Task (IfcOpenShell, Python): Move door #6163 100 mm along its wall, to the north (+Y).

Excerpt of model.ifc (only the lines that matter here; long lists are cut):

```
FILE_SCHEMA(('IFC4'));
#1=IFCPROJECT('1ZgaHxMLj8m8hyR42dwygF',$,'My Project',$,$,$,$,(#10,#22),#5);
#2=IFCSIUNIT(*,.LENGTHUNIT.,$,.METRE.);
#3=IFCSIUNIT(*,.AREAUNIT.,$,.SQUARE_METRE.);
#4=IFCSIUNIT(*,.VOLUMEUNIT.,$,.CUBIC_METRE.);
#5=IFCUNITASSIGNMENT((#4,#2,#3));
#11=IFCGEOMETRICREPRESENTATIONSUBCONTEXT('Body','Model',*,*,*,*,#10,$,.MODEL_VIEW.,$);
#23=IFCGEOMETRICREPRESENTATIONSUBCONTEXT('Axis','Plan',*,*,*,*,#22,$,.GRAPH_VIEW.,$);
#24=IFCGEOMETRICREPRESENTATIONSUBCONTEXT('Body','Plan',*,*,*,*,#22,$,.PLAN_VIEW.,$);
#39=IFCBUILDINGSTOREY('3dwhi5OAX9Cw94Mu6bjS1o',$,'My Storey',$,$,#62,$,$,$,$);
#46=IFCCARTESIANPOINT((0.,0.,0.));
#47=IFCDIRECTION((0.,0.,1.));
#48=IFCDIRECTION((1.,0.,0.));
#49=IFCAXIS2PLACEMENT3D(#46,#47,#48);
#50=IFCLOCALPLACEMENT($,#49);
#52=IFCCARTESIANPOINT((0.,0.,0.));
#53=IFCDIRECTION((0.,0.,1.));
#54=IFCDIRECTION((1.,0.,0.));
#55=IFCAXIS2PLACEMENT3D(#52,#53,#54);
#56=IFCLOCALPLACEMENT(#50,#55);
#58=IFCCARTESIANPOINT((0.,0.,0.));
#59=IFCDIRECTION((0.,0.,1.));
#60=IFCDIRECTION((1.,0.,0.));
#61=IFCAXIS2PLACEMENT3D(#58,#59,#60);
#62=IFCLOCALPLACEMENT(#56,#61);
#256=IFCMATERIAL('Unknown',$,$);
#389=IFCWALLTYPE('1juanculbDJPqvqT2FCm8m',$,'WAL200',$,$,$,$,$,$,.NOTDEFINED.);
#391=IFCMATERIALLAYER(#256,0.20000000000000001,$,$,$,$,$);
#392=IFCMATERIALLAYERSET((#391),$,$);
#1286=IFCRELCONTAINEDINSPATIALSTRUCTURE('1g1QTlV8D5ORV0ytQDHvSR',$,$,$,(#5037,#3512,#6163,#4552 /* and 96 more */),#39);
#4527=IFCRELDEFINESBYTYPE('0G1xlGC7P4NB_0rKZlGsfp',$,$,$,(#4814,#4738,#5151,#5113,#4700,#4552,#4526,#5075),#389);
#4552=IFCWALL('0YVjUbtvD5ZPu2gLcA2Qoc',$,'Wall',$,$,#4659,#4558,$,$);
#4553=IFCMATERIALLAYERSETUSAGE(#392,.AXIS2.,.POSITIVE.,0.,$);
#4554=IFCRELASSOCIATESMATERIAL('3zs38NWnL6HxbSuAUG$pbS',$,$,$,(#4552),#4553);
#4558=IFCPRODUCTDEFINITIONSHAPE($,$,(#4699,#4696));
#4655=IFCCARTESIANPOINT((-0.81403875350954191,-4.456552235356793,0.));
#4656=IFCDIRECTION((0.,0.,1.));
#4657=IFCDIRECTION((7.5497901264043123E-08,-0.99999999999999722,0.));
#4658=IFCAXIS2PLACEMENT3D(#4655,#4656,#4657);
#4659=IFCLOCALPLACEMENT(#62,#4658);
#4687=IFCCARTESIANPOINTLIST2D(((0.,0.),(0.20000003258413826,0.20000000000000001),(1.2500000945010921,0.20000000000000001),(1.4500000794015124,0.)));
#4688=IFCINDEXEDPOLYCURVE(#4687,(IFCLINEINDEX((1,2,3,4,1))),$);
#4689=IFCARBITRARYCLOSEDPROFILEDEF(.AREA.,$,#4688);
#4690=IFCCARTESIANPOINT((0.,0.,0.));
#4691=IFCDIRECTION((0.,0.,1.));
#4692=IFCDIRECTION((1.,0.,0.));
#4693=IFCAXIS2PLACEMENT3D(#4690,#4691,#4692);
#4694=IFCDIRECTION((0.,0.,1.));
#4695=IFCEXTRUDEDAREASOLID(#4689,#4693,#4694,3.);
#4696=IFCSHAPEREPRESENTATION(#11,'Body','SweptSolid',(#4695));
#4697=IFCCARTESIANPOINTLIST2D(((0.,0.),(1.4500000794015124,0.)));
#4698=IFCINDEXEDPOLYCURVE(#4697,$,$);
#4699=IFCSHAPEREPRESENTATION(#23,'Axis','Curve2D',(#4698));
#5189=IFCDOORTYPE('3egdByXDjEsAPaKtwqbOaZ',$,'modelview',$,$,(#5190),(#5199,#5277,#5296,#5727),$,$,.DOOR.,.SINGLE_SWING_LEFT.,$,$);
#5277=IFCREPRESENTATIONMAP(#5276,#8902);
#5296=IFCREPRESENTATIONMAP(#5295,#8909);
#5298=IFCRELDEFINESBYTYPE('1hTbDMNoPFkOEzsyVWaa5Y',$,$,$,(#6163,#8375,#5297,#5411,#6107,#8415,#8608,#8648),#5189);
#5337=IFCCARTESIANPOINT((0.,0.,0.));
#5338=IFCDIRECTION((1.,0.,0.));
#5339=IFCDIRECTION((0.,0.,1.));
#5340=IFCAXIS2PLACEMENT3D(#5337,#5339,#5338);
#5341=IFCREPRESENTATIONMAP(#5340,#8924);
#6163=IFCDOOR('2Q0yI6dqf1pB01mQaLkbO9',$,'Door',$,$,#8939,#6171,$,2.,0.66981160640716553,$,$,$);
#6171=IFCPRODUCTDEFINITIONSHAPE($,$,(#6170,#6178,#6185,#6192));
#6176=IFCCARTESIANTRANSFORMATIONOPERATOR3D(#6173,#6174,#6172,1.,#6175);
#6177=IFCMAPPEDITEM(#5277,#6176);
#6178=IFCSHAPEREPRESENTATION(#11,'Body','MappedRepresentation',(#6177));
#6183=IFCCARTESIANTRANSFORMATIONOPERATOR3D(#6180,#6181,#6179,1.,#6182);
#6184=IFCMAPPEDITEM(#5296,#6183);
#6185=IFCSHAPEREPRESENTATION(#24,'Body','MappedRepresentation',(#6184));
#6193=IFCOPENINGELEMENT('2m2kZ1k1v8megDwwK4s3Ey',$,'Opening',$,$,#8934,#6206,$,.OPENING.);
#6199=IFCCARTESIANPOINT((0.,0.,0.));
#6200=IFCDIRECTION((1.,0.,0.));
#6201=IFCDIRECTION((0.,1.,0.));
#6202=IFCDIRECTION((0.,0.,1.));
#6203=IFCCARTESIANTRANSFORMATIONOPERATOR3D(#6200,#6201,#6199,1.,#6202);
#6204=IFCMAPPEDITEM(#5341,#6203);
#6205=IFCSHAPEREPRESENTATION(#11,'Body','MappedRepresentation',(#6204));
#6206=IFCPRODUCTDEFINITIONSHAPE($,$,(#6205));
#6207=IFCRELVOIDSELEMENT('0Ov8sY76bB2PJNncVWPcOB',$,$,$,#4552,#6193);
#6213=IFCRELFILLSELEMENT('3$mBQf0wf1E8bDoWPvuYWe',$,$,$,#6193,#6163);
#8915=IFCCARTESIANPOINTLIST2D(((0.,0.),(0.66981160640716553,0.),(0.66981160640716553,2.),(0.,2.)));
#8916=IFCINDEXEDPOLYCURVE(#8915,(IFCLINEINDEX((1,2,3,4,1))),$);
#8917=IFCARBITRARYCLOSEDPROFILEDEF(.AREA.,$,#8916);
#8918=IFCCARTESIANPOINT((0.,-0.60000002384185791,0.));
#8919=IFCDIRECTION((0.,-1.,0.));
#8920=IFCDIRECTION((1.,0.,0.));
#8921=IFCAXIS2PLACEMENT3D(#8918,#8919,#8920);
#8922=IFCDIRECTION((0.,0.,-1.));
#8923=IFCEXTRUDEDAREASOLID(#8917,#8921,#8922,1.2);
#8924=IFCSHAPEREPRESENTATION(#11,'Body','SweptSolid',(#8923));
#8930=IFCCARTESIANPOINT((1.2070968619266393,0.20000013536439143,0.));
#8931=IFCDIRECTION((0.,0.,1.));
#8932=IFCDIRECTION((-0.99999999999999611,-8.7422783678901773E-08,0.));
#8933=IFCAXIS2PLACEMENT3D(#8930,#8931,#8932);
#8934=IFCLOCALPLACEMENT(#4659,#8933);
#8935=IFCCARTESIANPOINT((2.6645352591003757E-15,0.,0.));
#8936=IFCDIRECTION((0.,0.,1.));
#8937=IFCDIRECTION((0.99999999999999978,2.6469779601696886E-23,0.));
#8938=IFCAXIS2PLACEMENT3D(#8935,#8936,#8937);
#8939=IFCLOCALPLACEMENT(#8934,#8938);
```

```python
import ifcopenshell
import ifcopenshell.api.geometry
import ifcopenshell.util.placement
import ifcopenshell.util.unit

model = ifcopenshell.open("model.ifc")
unit_scale = ifcopenshell.util.unit.calculate_unit_scale(model)

door = model.by_id(6163)
opening = door.FillsVoids[0].RelatingOpeningElement
wall = opening.VoidsElements[0].RelatingBuildingElement

wall_matrix = ifcopenshell.util.placement.get_local_placement(wall.ObjectPlacement)
shift = wall_matrix[:3, 0] * -0.1 / unit_scale
before = ifcopenshell.util.placement.get_local_placement(door.ObjectPlacement)[:3, 3].copy()

# The door is placed relative to its opening, so it follows when the opening moves.
matrix = ifcopenshell.util.placement.get_local_placement(opening.ObjectPlacement)
matrix[:3, 3] += shift
ifcopenshell.api.geometry.edit_object_placement(
    model, product=opening, matrix=matrix, is_si=False, should_transform_children=True
)

after = ifcopenshell.util.placement.get_local_placement(door.ObjectPlacement)[:3, 3]
print("door moved by", (after - before).round(3) + 0.0)

model.write("model_updated.ifc")
```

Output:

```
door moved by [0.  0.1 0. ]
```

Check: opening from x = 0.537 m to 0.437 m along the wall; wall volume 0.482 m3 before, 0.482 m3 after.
